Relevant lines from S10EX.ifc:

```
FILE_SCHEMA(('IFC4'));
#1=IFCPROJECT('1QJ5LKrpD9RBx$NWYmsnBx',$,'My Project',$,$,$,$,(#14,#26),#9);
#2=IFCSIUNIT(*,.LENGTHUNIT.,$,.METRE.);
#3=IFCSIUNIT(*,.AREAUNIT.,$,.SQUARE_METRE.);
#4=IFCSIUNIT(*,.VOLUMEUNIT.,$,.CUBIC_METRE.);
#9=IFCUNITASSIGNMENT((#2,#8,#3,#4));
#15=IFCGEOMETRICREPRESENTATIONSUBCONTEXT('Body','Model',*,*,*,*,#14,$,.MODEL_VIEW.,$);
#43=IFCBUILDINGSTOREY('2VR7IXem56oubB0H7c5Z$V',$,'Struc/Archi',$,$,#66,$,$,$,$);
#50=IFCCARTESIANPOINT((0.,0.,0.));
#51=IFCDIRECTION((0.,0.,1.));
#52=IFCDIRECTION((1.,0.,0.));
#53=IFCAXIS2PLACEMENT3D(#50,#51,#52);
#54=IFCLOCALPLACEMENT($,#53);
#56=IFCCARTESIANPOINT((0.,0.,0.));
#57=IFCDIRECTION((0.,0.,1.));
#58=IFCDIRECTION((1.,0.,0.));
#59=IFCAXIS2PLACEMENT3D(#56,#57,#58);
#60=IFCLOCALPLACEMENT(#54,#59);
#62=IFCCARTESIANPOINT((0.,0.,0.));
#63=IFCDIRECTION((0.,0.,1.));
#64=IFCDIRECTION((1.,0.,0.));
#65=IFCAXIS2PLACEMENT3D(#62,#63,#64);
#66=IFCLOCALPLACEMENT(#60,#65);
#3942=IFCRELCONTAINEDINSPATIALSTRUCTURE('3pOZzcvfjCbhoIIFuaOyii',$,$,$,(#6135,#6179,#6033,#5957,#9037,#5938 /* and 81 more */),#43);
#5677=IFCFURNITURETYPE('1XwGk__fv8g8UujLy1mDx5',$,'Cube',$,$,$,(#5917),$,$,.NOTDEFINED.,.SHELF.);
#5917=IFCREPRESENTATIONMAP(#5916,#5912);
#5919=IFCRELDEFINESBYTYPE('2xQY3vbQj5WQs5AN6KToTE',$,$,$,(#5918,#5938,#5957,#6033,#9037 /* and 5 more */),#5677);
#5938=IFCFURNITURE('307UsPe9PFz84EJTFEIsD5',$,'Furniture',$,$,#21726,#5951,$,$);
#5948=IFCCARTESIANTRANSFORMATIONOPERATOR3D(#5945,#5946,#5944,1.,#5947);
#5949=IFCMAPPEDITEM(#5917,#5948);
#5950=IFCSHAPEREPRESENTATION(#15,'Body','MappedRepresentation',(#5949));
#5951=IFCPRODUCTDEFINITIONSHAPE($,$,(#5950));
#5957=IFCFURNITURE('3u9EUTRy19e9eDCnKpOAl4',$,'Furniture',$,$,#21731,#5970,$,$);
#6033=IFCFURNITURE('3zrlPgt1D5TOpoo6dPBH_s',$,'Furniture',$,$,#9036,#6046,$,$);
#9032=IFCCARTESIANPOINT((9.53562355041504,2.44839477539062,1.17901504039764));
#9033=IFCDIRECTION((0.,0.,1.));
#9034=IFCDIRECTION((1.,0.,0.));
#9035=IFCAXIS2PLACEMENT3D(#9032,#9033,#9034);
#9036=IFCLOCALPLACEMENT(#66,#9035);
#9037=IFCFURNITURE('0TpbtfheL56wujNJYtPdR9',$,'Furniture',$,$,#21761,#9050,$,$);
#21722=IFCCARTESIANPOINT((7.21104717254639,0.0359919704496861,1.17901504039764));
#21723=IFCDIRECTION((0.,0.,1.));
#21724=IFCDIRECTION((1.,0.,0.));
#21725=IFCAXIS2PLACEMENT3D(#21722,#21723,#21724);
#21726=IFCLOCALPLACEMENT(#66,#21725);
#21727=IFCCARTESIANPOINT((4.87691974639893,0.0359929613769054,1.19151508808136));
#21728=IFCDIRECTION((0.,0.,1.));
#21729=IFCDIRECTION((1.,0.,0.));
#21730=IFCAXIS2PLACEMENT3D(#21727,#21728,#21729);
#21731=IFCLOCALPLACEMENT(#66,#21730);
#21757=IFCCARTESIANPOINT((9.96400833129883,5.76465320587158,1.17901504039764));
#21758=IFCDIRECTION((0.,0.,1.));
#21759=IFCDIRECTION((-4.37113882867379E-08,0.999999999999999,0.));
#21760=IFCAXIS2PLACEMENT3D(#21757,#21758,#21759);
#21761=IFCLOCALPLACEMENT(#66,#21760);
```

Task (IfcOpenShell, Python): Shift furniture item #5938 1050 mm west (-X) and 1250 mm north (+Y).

```python
import ifcopenshell
import ifcopenshell.api.geometry
import ifcopenshell.util.placement

model = ifcopenshell.open("S10EX.ifc")

item = model.by_guid("307UsPe9PFz84EJTFEIsD5")
matrix = ifcopenshell.util.placement.get_local_placement(item.ObjectPlacement)
matrix[0, 3] -= 1.05
matrix[1, 3] += 1.25
ifcopenshell.api.geometry.edit_object_placement(model, product=item, matrix=matrix, is_si=False)

print(ifcopenshell.util.placement.get_local_placement(item.ObjectPlacement).round(3) + 0.0)

model.write("S10EX_edited.ifc")
```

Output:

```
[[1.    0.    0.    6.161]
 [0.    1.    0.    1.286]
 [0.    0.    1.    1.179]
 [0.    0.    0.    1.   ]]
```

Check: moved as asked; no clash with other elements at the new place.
